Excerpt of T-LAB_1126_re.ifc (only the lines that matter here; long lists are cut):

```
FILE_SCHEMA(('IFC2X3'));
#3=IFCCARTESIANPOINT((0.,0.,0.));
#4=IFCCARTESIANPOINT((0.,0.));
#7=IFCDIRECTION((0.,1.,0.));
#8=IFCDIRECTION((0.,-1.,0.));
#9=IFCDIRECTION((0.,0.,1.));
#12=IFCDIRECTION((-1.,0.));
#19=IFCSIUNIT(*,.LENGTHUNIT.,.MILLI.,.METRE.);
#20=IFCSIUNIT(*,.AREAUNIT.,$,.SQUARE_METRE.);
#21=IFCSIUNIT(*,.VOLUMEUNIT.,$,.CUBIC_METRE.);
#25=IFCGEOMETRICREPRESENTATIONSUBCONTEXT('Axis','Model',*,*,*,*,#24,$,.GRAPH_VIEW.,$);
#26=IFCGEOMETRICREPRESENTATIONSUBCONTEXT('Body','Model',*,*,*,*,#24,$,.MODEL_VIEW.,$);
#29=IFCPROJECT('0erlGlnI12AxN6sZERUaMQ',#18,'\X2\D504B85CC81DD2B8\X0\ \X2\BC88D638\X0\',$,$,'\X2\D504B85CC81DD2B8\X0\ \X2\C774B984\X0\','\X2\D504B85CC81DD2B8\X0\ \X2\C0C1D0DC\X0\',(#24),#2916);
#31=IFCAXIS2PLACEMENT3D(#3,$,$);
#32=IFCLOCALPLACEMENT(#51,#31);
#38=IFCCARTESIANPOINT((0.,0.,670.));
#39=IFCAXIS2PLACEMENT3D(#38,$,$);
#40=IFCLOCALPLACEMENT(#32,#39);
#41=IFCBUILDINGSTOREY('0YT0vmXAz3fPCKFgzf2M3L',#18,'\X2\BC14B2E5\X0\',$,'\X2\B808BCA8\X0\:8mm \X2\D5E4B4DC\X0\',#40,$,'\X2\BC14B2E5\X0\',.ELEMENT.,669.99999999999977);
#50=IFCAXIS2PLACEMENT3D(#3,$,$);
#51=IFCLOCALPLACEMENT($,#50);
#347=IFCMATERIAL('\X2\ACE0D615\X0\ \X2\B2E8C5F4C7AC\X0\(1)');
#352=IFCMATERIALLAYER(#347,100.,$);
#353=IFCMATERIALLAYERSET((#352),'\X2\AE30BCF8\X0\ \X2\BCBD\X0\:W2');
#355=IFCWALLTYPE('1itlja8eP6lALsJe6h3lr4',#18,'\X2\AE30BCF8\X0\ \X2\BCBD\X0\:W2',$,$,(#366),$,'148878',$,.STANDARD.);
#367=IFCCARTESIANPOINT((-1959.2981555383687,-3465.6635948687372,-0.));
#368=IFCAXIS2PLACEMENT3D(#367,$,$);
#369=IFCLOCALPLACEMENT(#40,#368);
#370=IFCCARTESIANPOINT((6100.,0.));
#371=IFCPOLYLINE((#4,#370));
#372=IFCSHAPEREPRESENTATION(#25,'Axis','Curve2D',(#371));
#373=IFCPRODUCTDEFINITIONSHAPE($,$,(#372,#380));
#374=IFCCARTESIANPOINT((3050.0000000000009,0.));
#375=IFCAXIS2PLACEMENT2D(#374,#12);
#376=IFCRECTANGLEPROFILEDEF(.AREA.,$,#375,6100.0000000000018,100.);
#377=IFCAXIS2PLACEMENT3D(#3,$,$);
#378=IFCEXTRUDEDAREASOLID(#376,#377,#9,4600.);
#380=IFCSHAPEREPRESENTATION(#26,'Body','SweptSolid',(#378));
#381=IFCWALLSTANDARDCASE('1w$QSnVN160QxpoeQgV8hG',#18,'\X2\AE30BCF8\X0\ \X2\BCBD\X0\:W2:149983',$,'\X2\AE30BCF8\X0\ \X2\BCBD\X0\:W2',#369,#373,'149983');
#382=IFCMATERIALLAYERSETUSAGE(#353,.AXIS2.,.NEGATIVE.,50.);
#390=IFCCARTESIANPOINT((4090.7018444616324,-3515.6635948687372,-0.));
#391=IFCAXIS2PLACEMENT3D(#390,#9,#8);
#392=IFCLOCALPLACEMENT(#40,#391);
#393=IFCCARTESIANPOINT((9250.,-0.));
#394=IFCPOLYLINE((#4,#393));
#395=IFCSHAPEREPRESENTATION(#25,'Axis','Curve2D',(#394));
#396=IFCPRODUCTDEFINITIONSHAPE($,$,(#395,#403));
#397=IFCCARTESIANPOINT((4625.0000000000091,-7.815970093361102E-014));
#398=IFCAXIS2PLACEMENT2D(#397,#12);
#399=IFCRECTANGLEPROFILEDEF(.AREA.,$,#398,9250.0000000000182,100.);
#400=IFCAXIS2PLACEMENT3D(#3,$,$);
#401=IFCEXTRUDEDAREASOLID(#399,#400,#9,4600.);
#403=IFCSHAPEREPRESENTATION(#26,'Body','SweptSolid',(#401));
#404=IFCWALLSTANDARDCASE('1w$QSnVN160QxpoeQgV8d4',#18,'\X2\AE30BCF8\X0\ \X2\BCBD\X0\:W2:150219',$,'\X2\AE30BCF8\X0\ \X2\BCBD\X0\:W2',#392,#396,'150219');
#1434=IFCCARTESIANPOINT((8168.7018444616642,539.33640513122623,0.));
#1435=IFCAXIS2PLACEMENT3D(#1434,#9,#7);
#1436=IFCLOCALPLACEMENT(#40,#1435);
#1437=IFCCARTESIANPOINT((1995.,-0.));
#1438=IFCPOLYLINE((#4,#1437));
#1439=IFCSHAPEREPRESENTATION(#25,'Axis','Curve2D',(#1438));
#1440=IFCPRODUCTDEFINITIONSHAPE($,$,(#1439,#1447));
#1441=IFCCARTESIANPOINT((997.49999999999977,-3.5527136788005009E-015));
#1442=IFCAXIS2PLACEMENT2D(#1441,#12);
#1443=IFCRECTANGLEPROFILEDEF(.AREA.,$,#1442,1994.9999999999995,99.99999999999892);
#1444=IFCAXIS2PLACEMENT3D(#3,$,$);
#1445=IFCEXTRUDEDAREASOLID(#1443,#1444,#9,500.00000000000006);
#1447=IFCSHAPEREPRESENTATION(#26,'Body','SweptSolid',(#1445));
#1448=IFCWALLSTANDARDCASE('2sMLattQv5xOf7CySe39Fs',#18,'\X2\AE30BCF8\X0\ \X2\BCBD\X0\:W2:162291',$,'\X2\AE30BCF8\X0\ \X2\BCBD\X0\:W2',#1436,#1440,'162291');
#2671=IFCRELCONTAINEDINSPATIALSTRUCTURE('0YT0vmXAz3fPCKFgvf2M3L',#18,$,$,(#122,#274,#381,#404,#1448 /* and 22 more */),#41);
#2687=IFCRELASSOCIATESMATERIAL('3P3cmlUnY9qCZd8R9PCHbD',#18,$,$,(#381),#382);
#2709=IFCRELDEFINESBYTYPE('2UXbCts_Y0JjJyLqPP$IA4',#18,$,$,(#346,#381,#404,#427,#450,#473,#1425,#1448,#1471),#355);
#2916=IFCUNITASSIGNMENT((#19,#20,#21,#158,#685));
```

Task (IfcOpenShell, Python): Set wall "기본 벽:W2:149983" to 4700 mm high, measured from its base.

```python
import ifcopenshell
import ifcopenshell.geom
import ifcopenshell.util.representation
import ifcopenshell.util.shape

model = ifcopenshell.open("T-LAB_1126_re.ifc")
settings = ifcopenshell.geom.settings()


def volume(element):
    """Net volume in cubic metres, openings subtracted."""
    shape = ifcopenshell.geom.create_shape(settings, element)
    return ifcopenshell.util.shape.get_volume(shape.geometry)


wall = model.by_guid("1w$QSnVN160QxpoeQgV8hG")
before = volume(wall)

body = ifcopenshell.util.representation.get_representation(wall, "Model", "Body")
solid = body.Items[0]
old_height = solid.Depth
solid.Depth = 4700.0
after = volume(wall)

print(f"height {old_height:g} -> {solid.Depth:g}, volume {before:.3f} -> {after:.3f} m3")

model.write("T-LAB_1126_re_edited.ifc")
```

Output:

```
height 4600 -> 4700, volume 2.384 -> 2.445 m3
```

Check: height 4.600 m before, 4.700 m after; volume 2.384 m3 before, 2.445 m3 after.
